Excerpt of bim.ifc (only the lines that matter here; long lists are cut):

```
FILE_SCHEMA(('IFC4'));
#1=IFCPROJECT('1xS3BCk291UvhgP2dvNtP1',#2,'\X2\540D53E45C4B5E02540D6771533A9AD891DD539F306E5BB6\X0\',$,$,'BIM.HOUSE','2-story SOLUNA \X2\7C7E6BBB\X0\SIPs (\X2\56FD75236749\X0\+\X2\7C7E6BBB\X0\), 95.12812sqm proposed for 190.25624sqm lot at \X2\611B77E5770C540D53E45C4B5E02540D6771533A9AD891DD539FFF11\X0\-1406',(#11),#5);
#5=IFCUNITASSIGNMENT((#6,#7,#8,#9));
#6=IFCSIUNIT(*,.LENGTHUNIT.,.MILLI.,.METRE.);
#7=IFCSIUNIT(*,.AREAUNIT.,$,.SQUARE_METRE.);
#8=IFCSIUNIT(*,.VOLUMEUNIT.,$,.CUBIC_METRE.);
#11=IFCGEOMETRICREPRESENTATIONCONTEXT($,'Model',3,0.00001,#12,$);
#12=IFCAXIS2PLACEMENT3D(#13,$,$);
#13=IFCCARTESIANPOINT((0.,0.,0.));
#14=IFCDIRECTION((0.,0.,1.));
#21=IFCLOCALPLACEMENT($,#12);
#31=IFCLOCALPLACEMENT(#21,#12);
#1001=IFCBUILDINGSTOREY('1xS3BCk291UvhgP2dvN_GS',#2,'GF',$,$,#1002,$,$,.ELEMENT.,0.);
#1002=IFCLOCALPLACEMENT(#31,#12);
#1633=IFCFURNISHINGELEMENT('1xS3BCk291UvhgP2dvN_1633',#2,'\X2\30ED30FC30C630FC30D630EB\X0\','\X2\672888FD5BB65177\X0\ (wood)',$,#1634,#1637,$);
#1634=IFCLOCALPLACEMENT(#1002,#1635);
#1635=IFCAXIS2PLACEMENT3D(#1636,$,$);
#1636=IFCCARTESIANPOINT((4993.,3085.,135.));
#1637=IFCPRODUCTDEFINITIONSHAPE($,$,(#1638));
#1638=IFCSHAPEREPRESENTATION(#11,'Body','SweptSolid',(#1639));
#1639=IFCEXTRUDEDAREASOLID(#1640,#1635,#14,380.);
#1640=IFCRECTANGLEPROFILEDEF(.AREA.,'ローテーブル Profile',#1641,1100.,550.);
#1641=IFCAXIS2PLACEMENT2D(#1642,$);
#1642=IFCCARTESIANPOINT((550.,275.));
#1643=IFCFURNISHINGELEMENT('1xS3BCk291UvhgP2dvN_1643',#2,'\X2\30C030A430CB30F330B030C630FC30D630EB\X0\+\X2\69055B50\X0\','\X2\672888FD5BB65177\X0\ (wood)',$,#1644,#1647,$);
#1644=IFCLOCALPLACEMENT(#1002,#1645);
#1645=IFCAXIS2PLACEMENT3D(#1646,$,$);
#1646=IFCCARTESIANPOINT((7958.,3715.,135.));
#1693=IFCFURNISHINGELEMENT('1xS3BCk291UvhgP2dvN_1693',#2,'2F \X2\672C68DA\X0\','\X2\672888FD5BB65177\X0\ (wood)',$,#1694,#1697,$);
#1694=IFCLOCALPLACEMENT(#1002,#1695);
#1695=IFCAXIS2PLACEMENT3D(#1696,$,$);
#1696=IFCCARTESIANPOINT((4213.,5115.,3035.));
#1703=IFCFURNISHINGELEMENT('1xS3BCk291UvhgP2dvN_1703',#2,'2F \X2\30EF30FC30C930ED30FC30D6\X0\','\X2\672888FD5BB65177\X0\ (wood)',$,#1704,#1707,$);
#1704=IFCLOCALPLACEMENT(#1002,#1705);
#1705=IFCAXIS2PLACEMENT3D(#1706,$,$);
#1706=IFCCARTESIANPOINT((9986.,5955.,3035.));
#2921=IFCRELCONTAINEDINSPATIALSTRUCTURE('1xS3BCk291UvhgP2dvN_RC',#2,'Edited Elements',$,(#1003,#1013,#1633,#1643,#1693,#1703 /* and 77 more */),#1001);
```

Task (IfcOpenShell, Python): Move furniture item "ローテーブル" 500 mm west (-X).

```python
import ifcopenshell
import ifcopenshell.api.geometry
import ifcopenshell.util.placement

model = ifcopenshell.open("bim.ifc")

item = model.by_guid("1xS3BCk291UvhgP2dvN_1633")
matrix = ifcopenshell.util.placement.get_local_placement(item.ObjectPlacement)
matrix[0, 3] -= 500.0
ifcopenshell.api.geometry.edit_object_placement(model, product=item, matrix=matrix, is_si=False)

print(ifcopenshell.util.placement.get_local_placement(item.ObjectPlacement).round(3) + 0.0)

model.write("bim_updated.ifc")
```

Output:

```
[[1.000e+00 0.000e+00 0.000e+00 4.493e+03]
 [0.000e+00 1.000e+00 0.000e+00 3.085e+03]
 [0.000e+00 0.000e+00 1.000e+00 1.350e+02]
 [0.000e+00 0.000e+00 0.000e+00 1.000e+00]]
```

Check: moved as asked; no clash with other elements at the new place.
